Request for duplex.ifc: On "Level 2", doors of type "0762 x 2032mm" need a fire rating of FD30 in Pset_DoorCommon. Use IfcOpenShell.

First a look at what the model holds.

```python
import ifcopenshell
import ifcopenshell.util.element

model = ifcopenshell.open("duplex.ifc")
print(model.schema)
storey = next(s for s in model.by_type("IfcBuildingStorey") if s.Name == "Level 2")
doors = [e for e in ifcopenshell.util.element.get_decomposition(storey) if e.is_a("IfcDoor")]
seen = {}
for e in doors:
    element_type = ifcopenshell.util.element.get_type(e)
    key = (element_type.Name if element_type != e and element_type else None, ifcopenshell.util.element.get_pset(e, "Pset_DoorCommon", "FireRating"))
    seen[key] = seen.get(key, 0) + 1
for (name, value), count in sorted(seen.items(), key=str):
    print(count, "x", name, "|", value)
```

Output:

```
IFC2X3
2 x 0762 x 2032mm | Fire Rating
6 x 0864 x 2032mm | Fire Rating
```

```python
import ifcopenshell
import ifcopenshell.api.pset
import ifcopenshell.util.element

model = ifcopenshell.open("duplex.ifc")

storey = next(s for s in model.by_type("IfcBuildingStorey") if s.Name == "Level 2")
doors = [e for e in ifcopenshell.util.element.get_decomposition(storey) if e.is_a("IfcDoor")]

count = 0
for e in doors:
    element_type = ifcopenshell.util.element.get_type(e)
    if element_type in (None, e) or element_type.Name != "0762 x 2032mm":
        continue
    # add_pset returns the element's existing set when there is one.
    pset = ifcopenshell.api.pset.add_pset(model, product=e, name="Pset_DoorCommon")
    ifcopenshell.api.pset.edit_pset(model, pset=pset, properties={"FireRating": "FD30"})
    count += 1

print(count, "doors updated")

model.write("duplex_edited.ifc")
```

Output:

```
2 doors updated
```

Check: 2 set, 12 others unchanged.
